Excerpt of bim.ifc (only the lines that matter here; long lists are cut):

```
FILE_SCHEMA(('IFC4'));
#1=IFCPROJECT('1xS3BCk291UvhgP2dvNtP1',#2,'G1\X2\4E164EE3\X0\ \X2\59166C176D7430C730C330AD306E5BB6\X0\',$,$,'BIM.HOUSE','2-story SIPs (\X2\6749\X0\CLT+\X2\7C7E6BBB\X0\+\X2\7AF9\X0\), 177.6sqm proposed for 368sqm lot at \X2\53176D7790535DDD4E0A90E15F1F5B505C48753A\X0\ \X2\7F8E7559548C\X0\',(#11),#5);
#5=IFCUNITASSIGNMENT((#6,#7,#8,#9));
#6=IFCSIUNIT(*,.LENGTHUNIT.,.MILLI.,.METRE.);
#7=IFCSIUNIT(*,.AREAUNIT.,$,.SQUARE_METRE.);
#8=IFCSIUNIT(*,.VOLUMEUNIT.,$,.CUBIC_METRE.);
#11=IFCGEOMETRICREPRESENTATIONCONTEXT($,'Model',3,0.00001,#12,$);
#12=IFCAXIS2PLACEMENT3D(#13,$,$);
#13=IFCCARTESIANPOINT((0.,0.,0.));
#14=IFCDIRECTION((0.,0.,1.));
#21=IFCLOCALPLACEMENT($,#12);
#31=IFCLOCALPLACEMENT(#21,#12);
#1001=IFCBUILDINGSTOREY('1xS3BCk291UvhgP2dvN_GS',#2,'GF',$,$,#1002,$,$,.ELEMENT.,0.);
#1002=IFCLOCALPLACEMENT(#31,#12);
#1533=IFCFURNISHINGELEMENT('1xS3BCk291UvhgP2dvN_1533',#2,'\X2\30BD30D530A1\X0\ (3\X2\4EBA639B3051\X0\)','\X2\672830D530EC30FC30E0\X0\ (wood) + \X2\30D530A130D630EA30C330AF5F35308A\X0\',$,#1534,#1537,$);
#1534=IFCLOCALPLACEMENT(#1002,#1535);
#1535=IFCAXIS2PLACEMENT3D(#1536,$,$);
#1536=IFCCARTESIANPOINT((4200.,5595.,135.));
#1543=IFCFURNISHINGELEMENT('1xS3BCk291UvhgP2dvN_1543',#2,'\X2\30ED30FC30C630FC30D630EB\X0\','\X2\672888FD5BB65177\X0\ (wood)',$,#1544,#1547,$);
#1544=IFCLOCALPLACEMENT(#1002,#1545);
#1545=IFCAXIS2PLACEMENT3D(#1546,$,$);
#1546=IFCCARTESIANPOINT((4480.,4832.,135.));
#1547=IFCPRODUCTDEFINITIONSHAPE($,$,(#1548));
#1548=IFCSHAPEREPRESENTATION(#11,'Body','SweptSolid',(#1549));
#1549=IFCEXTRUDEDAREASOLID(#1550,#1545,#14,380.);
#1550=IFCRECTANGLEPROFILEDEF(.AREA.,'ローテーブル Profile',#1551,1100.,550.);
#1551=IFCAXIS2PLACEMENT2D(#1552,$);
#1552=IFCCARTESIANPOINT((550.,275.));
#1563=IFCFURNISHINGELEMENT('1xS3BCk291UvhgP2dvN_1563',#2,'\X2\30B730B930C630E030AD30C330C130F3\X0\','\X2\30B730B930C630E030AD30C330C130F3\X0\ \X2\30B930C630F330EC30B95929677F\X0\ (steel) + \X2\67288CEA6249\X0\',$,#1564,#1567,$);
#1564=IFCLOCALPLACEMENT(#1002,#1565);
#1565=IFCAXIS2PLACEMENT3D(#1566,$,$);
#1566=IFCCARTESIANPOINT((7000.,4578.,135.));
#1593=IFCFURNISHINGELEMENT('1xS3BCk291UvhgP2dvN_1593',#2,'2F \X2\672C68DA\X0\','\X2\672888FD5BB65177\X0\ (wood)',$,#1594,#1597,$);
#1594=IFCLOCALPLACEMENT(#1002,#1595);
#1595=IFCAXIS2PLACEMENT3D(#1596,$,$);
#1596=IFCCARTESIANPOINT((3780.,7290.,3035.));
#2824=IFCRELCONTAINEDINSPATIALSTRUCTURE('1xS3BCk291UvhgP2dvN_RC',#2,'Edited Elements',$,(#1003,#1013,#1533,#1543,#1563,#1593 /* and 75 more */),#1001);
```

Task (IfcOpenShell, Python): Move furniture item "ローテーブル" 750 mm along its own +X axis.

```python
import ifcopenshell
import ifcopenshell.api.geometry
import ifcopenshell.util.placement
import ifcopenshell.util.unit

model = ifcopenshell.open("bim.ifc")
unit_scale = ifcopenshell.util.unit.calculate_unit_scale(model)

item = model.by_id(1543)
matrix = ifcopenshell.util.placement.get_local_placement(item.ObjectPlacement)
matrix[:3, 3] += matrix[:3, 0] * 0.75 / unit_scale
ifcopenshell.api.geometry.edit_object_placement(model, product=item, matrix=matrix, is_si=False)

print(ifcopenshell.util.placement.get_local_placement(item.ObjectPlacement).round(3) + 0.0)

model.write("bim_updated.ifc")
```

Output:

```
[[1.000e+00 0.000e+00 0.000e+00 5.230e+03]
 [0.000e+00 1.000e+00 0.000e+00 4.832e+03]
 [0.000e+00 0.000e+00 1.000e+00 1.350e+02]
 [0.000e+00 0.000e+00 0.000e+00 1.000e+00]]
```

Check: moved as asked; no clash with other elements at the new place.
